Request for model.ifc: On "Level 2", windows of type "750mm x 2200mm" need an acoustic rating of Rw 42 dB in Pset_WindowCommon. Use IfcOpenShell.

First a look at what the model holds.

```python
import ifcopenshell
import ifcopenshell.util.element

model = ifcopenshell.open("model.ifc")
print(model.schema)
storey = next(s for s in model.by_type("IfcBuildingStorey") if s.Name == "Level 2")
windows = [e for e in ifcopenshell.util.element.get_decomposition(storey) if e.is_a("IfcWindow")]
seen = {}
for e in windows:
    element_type = ifcopenshell.util.element.get_type(e)
    key = (element_type.Name if element_type != e and element_type else None, ifcopenshell.util.element.get_pset(e, "Pset_WindowCommon", "AcousticRating"))
    seen[key] = seen.get(key, 0) + 1
for (name, value), count in sorted(seen.items(), key=str):
    print(count, "x", name, "|", value)
```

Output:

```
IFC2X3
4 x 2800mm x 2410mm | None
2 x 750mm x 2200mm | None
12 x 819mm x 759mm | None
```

```python
import ifcopenshell
import ifcopenshell.api.pset
import ifcopenshell.util.element

model = ifcopenshell.open("model.ifc")

storey = next(s for s in model.by_type("IfcBuildingStorey") if s.Name == "Level 2")
windows = [e for e in ifcopenshell.util.element.get_decomposition(storey) if e.is_a("IfcWindow")]

count = 0
for e in windows:
    element_type = ifcopenshell.util.element.get_type(e)
    if element_type in (None, e) or element_type.Name != "750mm x 2200mm":
        continue
    # add_pset returns the element's existing set when there is one.
    pset = ifcopenshell.api.pset.add_pset(model, product=e, name="Pset_WindowCommon")
    ifcopenshell.api.pset.edit_pset(model, pset=pset, properties={"AcousticRating": "Rw 42 dB"})
    count += 1

print(count, "windows updated")

model.write("model_rev.ifc")
```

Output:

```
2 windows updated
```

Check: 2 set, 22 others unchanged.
